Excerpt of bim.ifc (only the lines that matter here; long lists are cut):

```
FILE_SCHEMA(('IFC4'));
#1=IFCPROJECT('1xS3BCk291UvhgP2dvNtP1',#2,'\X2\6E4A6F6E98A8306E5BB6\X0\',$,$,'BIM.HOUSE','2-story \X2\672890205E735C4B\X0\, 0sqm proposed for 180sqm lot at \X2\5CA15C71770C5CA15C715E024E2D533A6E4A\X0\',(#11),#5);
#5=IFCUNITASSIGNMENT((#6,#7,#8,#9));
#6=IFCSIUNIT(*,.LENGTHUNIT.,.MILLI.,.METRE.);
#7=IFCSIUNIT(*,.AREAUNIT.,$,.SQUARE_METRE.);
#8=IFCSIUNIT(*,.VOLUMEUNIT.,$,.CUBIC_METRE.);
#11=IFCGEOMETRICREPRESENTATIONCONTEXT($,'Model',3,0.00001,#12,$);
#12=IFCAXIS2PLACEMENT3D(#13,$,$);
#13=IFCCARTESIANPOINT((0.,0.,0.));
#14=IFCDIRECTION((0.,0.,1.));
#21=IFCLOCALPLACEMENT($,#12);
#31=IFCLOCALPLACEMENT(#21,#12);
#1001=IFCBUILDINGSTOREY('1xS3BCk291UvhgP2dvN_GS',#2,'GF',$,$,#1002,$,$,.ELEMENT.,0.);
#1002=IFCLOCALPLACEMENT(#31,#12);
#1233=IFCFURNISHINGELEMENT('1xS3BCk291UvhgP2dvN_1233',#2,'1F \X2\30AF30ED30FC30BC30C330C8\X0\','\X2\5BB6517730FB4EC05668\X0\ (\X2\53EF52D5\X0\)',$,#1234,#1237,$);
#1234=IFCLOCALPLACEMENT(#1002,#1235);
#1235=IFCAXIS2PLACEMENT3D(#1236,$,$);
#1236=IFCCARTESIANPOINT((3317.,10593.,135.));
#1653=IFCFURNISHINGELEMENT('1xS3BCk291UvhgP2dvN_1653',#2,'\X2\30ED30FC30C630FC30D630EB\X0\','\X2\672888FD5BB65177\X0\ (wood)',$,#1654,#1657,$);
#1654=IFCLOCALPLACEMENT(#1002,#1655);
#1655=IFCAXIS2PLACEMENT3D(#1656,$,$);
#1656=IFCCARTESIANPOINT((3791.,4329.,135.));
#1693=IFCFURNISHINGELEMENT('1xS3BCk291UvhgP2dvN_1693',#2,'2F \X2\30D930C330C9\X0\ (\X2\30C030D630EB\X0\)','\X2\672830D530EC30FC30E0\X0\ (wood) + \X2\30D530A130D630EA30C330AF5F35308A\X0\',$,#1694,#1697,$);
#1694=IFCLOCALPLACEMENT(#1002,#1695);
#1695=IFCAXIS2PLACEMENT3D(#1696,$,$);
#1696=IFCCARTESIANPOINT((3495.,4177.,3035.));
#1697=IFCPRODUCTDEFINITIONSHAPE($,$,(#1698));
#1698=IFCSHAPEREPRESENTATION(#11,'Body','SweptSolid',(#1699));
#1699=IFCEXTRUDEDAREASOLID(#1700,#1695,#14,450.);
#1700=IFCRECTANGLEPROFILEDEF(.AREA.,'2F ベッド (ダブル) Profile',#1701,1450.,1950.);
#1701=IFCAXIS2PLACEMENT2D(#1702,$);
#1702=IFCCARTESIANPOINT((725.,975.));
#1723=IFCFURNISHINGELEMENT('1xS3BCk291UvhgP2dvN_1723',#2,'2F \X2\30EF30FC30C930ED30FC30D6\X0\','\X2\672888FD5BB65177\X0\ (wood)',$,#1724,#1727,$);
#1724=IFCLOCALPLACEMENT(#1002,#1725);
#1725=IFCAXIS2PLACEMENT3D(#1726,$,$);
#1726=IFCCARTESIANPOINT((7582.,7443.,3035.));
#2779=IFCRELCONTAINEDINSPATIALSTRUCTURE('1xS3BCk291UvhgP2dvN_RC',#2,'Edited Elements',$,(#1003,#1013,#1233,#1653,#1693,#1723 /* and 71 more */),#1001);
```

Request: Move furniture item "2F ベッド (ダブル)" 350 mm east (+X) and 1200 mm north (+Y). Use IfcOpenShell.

```python
import ifcopenshell
import ifcopenshell.api.geometry
import ifcopenshell.util.placement

model = ifcopenshell.open("bim.ifc")

item = model.by_id(1693)
matrix = ifcopenshell.util.placement.get_local_placement(item.ObjectPlacement)
matrix[0, 3] += 350.0
matrix[1, 3] += 1200.0
ifcopenshell.api.geometry.edit_object_placement(model, product=item, matrix=matrix, is_si=False)

print(ifcopenshell.util.placement.get_local_placement(item.ObjectPlacement).round(3) + 0.0)

model.write("bim_edited.ifc")
```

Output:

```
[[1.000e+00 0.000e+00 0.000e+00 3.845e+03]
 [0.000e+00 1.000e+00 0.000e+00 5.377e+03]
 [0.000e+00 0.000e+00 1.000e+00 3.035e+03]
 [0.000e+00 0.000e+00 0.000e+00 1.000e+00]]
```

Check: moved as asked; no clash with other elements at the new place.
